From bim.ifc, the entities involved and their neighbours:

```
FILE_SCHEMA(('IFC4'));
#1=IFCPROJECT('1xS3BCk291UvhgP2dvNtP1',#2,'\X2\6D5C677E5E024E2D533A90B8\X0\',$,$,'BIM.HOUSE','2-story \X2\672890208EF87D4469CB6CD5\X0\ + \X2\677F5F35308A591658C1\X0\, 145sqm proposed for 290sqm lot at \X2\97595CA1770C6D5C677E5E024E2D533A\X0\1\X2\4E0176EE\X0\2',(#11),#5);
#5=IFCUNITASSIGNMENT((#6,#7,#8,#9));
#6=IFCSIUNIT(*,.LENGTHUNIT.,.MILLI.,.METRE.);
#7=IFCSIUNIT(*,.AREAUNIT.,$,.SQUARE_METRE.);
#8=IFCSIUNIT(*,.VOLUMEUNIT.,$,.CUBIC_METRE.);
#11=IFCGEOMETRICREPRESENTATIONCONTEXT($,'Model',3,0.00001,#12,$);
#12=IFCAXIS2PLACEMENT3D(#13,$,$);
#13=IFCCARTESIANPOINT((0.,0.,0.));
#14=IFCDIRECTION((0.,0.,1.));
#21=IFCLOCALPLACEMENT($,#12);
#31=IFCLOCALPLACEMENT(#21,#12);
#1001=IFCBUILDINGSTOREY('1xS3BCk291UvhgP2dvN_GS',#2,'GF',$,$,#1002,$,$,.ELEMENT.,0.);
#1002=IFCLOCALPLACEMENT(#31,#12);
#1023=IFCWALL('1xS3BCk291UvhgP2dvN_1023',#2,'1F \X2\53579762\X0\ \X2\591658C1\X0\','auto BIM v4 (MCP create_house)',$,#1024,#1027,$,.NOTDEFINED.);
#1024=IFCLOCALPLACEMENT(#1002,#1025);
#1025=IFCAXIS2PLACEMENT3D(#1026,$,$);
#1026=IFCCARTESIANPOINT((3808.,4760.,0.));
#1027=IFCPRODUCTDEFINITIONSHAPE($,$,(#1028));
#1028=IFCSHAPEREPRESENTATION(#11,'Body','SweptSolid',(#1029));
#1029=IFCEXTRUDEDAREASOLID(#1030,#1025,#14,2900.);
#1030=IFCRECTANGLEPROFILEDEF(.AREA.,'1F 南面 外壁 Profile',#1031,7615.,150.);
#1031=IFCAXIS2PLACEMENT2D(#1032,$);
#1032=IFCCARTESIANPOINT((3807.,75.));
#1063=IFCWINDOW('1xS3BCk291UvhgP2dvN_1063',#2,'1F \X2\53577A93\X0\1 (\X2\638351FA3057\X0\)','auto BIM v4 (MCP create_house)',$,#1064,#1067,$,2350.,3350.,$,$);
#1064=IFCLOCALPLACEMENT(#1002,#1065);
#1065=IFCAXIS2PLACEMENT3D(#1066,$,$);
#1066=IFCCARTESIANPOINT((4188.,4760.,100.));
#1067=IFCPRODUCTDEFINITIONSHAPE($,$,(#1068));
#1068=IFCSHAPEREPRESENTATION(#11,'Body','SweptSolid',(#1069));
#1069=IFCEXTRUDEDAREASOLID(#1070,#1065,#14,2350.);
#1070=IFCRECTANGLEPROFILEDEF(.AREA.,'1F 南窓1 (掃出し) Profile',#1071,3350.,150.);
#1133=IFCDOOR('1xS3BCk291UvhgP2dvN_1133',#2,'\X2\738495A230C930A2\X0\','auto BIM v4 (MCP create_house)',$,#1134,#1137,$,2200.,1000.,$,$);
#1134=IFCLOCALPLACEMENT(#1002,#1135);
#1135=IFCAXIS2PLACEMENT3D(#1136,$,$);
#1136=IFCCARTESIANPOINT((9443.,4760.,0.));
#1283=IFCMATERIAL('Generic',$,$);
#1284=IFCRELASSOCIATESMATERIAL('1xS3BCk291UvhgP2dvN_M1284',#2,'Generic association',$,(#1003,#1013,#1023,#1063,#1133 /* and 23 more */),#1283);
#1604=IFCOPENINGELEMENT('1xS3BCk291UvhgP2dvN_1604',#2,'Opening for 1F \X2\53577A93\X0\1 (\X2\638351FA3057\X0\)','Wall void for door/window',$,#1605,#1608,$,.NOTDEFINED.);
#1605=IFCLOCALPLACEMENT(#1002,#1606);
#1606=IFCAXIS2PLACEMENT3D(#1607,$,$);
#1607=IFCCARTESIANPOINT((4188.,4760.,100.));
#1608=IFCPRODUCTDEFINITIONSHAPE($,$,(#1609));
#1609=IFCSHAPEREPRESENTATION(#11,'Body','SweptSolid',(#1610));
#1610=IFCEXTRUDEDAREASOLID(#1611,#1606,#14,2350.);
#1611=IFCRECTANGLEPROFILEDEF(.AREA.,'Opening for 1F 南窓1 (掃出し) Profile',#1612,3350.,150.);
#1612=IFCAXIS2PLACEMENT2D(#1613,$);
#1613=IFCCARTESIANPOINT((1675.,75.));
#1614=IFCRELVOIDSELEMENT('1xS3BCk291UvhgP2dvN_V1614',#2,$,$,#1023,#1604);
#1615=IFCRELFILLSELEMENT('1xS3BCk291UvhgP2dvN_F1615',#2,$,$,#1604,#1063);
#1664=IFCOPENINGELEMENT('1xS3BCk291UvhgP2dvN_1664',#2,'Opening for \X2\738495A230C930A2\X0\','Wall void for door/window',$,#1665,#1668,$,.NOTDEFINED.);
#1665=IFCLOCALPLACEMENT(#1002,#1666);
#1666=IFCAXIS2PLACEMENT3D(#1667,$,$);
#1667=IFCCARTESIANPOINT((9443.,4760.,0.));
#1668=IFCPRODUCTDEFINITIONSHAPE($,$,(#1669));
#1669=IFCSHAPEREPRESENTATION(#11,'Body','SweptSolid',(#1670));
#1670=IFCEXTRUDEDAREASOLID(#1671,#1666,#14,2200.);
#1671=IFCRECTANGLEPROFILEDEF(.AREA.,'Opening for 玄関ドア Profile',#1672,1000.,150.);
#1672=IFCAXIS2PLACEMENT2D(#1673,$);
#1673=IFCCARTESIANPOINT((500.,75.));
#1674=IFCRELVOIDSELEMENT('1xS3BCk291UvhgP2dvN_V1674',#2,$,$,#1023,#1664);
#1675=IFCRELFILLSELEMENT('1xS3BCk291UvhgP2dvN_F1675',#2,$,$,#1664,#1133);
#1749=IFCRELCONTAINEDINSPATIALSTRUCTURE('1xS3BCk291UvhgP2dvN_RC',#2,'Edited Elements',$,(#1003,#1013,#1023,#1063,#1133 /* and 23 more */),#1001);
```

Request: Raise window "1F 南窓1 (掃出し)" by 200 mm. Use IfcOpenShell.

```python
import numpy as np
import ifcopenshell
import ifcopenshell.api.geometry
import ifcopenshell.util.placement
import ifcopenshell.util.unit

model = ifcopenshell.open("bim.ifc")
unit_scale = ifcopenshell.util.unit.calculate_unit_scale(model)

window = model.by_guid("1xS3BCk291UvhgP2dvN_1063")
opening = window.FillsVoids[0].RelatingOpeningElement
dz = 200.0

shift = np.array([0.0, 0.0, dz])
# The window is not placed relative to its opening, so move both.
for product in (opening, window):
    matrix = ifcopenshell.util.placement.get_local_placement(product.ObjectPlacement)
    matrix[:3, 3] += shift
    ifcopenshell.api.geometry.edit_object_placement(model, product=product, matrix=matrix, is_si=False)

print(f"moved by {dz * unit_scale:+.3f} m")

model.write("bim_v2.ifc")
```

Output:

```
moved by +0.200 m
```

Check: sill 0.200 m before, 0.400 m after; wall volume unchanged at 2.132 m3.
